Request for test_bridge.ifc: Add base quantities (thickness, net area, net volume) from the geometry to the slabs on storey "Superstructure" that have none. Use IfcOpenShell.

First a look at what the model holds.

```python
import ifcopenshell
import ifcopenshell.util.element
import ifcopenshell.util.unit

model = ifcopenshell.open("test_bridge.ifc")
print(model.schema)
for unit_type in ("LENGTHUNIT", "AREAUNIT", "VOLUMEUNIT"):
    print(unit_type, ifcopenshell.util.unit.calculate_unit_scale(model, unit_type))
storey = next(s for s in model.by_type("IfcBuildingStorey") if s.Name == "Superstructure")
slabs = [e for e in ifcopenshell.util.element.get_decomposition(storey) if e.is_a("IfcSlab")]
for e in sorted(slabs, key=lambda e: e.id()):
    print(e.id(), e.is_a(), e.Name, list(ifcopenshell.util.element.get_psets(e, qtos_only=True)), sep=" | ")
```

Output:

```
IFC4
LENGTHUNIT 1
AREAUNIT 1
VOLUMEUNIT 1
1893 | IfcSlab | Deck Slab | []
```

```python
import ifcopenshell
import ifcopenshell.api.pset
import ifcopenshell.geom
import ifcopenshell.util.element
import ifcopenshell.util.shape
import ifcopenshell.util.unit

model = ifcopenshell.open("test_bridge.ifc")
unit_scale = ifcopenshell.util.unit.calculate_unit_scale(model)
area_scale = ifcopenshell.util.unit.calculate_unit_scale(model, "AREAUNIT")
volume_scale = ifcopenshell.util.unit.calculate_unit_scale(model, "VOLUMEUNIT")
settings = ifcopenshell.geom.settings()

storey = next(s for s in model.by_type("IfcBuildingStorey") if s.Name == "Superstructure")
slabs = [e for e in ifcopenshell.util.element.get_decomposition(storey) if e.is_a("IfcSlab")]

for e in sorted(slabs, key=lambda e: e.id()):
    if ifcopenshell.util.element.get_psets(e, qtos_only=True, should_inherit=False):
        continue
    # Geometry comes back in metres, in the element's own axes.
    shape = ifcopenshell.geom.create_shape(settings, e)
    values = {
        "Width": ifcopenshell.util.shape.get_z(shape.geometry) / unit_scale,
        "NetArea": ifcopenshell.util.shape.get_footprint_area(shape.geometry) / area_scale,
        "NetVolume": ifcopenshell.util.shape.get_volume(shape.geometry) / volume_scale,
    }
    qto = ifcopenshell.api.pset.add_qto(model, product=e, name="Qto_SlabBaseQuantities")
    ifcopenshell.api.pset.edit_qto(model, qto=qto, properties=values)
    print(e.id(), {k: round(v, 3) for k, v in values.items()})

model.write("test_bridge_edited.ifc")
```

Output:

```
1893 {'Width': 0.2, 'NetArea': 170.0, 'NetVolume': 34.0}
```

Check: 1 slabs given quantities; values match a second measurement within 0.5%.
